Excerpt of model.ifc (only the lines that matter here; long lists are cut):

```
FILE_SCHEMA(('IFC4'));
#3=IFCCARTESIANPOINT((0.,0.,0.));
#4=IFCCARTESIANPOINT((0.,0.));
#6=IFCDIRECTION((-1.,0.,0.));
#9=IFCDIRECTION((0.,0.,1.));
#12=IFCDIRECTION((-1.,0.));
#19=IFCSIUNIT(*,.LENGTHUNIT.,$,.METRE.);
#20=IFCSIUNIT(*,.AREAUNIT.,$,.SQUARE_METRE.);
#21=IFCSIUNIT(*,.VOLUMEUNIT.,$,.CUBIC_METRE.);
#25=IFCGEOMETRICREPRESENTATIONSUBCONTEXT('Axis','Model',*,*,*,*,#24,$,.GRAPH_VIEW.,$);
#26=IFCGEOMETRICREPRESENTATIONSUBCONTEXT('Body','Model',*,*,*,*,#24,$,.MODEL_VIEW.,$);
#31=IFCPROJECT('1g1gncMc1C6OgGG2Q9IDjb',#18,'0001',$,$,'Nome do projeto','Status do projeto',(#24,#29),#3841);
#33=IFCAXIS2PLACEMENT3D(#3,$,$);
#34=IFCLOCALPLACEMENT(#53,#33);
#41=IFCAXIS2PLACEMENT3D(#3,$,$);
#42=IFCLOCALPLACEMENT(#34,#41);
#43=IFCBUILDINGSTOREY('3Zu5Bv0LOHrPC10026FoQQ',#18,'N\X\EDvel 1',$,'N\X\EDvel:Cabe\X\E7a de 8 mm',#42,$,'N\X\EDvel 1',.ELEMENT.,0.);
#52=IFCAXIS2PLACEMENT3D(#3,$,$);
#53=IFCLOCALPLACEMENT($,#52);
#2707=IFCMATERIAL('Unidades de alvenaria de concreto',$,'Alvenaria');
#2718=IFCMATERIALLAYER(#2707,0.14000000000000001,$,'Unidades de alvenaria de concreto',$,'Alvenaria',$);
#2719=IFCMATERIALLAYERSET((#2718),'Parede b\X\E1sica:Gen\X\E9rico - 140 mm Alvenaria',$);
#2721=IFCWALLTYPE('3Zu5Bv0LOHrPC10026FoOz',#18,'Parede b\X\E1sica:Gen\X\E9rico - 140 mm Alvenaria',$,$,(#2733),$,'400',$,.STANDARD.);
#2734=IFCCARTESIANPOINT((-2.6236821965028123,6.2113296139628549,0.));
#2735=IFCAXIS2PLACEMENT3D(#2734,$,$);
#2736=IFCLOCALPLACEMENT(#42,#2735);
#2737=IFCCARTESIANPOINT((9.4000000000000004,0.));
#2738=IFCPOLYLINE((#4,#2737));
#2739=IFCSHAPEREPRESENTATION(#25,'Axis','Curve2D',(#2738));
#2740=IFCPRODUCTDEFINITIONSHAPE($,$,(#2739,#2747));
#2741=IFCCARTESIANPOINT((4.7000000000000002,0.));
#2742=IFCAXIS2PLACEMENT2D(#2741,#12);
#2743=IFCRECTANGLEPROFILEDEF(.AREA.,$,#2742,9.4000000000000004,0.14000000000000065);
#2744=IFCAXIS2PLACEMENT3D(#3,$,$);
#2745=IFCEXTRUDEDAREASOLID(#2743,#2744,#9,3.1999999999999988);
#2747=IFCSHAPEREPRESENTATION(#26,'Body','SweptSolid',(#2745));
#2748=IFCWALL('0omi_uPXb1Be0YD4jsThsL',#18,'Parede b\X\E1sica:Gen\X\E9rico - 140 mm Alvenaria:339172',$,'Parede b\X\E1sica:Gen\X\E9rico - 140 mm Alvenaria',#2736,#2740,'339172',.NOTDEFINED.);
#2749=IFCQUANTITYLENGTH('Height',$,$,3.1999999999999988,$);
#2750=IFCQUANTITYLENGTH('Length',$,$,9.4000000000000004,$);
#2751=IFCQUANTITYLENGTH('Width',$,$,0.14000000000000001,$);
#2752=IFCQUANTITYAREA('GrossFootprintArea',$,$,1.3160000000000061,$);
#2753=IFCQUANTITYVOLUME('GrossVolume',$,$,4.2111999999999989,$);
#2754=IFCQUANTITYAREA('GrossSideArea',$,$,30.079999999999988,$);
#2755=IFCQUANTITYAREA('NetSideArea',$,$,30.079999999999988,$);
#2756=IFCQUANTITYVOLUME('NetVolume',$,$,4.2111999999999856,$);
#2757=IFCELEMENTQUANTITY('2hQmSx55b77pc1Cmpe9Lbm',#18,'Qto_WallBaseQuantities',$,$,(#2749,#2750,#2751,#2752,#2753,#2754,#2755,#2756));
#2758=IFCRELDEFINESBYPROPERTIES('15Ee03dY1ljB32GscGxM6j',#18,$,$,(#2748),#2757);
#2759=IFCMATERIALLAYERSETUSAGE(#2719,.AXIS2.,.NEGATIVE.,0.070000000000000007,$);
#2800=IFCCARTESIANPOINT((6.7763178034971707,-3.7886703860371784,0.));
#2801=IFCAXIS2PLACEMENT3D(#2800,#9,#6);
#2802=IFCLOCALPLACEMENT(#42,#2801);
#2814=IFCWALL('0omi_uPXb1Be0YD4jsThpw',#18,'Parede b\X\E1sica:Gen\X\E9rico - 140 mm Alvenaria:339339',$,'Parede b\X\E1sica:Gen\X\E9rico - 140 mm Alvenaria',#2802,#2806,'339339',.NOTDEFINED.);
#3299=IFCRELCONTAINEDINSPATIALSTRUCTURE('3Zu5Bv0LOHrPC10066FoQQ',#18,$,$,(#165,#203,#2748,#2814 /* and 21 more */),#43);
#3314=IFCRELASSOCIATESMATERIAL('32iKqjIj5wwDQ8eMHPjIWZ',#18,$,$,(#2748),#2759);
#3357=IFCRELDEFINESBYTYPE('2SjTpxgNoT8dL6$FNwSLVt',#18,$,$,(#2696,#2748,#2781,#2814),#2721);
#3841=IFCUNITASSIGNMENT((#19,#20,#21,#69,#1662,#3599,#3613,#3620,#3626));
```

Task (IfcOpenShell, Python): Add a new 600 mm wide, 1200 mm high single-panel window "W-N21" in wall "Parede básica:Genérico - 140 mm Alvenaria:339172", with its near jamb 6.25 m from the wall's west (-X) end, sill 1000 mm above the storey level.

```python
import numpy as np
import ifcopenshell
import ifcopenshell.api.feature
import ifcopenshell.api.geometry
import ifcopenshell.api.pset
import ifcopenshell.api.root
import ifcopenshell.api.spatial
import ifcopenshell.geom
import ifcopenshell.util.element
import ifcopenshell.util.placement
import ifcopenshell.util.representation
import ifcopenshell.util.shape
import ifcopenshell.util.unit

model = ifcopenshell.open("model.ifc")
unit_scale = ifcopenshell.util.unit.calculate_unit_scale(model)
area_scale = ifcopenshell.util.unit.calculate_unit_scale(model, "AREAUNIT")
volume_scale = ifcopenshell.util.unit.calculate_unit_scale(model, "VOLUMEUNIT")
settings = ifcopenshell.geom.settings()


def volume(element):
    """Net volume in cubic metres, openings subtracted."""
    shape = ifcopenshell.geom.create_shape(settings, element)
    return ifcopenshell.util.shape.get_volume(shape.geometry)


wall = model.by_id(2748)
storey = ifcopenshell.util.element.get_container(wall, ifc_class="IfcBuildingStorey")
context = ifcopenshell.util.representation.get_context(model, "Model", "Body", "MODEL_VIEW")
before = volume(wall)

width, height, from_end, sill = 0.6, 1.2, 6.25, 1  # metres

# The wall runs along its own X axis, and the end named is its -X end.
wall_shape = ifcopenshell.geom.create_shape(settings, wall)
x, y, z = ifcopenshell.util.shape.get_vertices(wall_shape.geometry).T
start = x.min() + from_end
face, thickness = float(y.min()), float(y.max() - y.min())
wall_matrix = ifcopenshell.util.placement.get_local_placement(wall.ObjectPlacement)
level = ifcopenshell.util.placement.get_local_placement(storey.ObjectPlacement)[2, 3]


def in_wall(x, y):
    """Placement at x, y metres in the wall's axes, at sill height."""
    matrix = wall_matrix.copy()
    matrix[:, 3] = wall_matrix @ np.array([x / unit_scale, y / unit_scale, 0.0, 1.0])
    matrix[2, 3] = level + sill / unit_scale
    return matrix


# Opening: a box that overshoots both wall faces by 50 mm.
opening = ifcopenshell.api.root.create_entity(model, ifc_class="IfcOpeningElement", predefined_type="OPENING")
box = ifcopenshell.api.geometry.add_wall_representation(
    model, context=context, length=width, height=height, thickness=thickness + 0.1
)
ifcopenshell.api.geometry.assign_representation(model, product=opening, representation=box)
ifcopenshell.api.geometry.edit_object_placement(model, product=opening, matrix=in_wall(start, face - 0.05), is_si=False)
ifcopenshell.api.feature.add_feature(model, feature=opening, element=wall)

window = ifcopenshell.api.root.create_entity(model, ifc_class="IfcWindow", name="W-N21", predefined_type="WINDOW")
window.OverallWidth, window.OverallHeight = width / unit_scale, height / unit_scale
window.PartitioningType = "SINGLE_PANEL"
body = ifcopenshell.api.geometry.add_window_representation(
    model,
    context=context,
    overall_width=window.OverallWidth,
    overall_height=window.OverallHeight,
    partition_type="SINGLE_PANEL",
)
ifcopenshell.api.geometry.assign_representation(model, product=window, representation=body)
ifcopenshell.api.spatial.assign_container(model, products=[window], relating_structure=storey)
ifcopenshell.api.feature.add_filling(model, opening=opening, element=window)

# Centre the window in the wall's thickness.
ifcopenshell.api.geometry.edit_object_placement(model, product=window, matrix=in_wall(start, face), is_si=False)
window_shape = ifcopenshell.geom.create_shape(settings, window)
depth = ifcopenshell.util.shape.get_vertices(window_shape.geometry)[:, 1]
offset = face + thickness / 2 - (depth.min() + depth.max()) / 2
ifcopenshell.api.geometry.edit_object_placement(model, product=window, matrix=in_wall(start, offset), is_si=False)

after = volume(wall)

# Update the wall's stored quantities.
qto = model.by_id(ifcopenshell.util.element.get_pset(wall, "Qto_WallBaseQuantities", should_inherit=False)["id"])
ifcopenshell.api.pset.edit_qto(model, qto=qto, properties={
    "NetSideArea": after / thickness / area_scale,
    "NetVolume": after / volume_scale,
})

print(f"wall volume {before:.3f} -> {after:.3f} m3")

model.write("model-out.ifc")
```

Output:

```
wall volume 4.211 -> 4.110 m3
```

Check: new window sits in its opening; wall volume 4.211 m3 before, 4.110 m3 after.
